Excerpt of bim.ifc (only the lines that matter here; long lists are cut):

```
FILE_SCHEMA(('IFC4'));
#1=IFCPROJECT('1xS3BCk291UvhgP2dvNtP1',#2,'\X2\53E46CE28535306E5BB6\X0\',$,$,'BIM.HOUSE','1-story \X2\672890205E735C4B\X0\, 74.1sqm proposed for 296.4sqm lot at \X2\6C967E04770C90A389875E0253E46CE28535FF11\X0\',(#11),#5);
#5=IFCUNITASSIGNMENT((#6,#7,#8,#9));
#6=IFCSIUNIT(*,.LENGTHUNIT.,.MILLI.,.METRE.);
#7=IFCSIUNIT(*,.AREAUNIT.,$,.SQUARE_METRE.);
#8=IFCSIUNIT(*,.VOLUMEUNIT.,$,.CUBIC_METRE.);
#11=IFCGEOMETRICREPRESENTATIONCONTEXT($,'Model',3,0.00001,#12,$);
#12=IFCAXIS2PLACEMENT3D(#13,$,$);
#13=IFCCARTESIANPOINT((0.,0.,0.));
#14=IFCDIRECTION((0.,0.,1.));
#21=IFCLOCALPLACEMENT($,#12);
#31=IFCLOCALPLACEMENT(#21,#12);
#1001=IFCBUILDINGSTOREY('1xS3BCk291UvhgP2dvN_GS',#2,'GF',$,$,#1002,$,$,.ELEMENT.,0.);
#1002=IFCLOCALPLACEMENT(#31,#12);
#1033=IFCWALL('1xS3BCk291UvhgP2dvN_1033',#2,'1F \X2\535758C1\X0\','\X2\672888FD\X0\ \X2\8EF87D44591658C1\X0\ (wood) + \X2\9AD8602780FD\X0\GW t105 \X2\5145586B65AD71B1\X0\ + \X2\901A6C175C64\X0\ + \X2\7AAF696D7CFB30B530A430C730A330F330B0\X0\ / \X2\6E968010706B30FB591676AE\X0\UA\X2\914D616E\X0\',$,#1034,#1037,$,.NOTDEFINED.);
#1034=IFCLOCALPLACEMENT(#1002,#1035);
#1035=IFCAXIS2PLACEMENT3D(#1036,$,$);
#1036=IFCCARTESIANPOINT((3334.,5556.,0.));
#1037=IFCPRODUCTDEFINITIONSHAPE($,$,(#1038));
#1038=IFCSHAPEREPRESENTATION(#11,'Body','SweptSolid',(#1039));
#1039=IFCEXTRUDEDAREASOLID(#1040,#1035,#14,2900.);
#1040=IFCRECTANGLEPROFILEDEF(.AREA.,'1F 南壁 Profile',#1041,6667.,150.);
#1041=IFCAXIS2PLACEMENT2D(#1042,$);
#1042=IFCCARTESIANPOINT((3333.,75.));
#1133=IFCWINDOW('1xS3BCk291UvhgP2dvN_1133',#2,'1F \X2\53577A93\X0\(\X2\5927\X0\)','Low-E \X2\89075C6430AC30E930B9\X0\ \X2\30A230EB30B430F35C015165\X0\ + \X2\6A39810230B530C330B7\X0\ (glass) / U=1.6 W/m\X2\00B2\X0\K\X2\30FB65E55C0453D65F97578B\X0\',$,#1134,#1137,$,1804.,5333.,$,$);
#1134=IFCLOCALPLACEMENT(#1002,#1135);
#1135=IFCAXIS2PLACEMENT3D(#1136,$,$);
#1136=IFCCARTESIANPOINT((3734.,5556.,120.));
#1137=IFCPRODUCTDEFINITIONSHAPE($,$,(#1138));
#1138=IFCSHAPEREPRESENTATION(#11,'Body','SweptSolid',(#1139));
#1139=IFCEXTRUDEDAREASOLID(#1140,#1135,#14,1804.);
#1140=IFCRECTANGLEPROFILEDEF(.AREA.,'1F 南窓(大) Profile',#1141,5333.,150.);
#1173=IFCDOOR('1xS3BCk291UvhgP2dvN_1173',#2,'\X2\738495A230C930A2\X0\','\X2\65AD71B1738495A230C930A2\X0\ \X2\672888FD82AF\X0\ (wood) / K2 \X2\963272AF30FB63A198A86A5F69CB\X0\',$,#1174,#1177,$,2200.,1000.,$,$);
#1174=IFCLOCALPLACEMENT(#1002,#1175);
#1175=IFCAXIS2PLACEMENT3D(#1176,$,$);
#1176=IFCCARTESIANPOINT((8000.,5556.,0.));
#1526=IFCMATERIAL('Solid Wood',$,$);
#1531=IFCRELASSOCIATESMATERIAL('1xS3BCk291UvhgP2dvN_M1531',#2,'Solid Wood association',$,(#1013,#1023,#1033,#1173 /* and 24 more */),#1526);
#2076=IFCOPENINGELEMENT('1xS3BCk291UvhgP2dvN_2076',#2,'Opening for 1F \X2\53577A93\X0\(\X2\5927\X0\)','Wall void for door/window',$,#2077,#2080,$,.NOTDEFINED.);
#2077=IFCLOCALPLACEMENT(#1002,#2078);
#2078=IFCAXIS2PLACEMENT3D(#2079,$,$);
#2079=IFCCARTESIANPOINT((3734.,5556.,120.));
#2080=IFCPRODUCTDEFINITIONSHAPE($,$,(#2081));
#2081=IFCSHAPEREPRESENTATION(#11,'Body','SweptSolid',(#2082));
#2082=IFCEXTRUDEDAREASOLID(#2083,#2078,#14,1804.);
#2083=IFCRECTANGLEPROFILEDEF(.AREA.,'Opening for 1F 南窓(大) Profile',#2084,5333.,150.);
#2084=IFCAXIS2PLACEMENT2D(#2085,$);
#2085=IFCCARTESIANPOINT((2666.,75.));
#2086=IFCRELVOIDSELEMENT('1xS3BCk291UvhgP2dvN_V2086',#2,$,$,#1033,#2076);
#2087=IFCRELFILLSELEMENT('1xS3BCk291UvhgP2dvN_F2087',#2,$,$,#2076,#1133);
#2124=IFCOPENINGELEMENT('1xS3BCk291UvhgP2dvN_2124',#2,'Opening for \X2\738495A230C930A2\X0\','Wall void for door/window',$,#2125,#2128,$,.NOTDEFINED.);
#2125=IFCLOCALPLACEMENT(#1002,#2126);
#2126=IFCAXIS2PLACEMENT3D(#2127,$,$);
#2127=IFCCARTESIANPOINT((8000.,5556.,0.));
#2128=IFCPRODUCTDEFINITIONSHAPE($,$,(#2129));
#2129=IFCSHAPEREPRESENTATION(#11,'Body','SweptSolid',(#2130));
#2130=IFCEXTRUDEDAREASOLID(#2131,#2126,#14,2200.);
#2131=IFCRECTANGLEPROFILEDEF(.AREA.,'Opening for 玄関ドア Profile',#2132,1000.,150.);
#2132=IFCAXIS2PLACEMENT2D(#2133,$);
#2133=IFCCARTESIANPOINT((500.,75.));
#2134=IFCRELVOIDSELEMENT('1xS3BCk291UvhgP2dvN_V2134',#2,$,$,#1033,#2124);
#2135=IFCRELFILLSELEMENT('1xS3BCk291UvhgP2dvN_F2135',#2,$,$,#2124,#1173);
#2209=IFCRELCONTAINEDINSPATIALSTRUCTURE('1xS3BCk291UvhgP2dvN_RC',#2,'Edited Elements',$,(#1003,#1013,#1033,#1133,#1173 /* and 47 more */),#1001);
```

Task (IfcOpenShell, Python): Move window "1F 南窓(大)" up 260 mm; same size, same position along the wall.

```python
import numpy as np
import ifcopenshell
import ifcopenshell.api.geometry
import ifcopenshell.util.placement
import ifcopenshell.util.unit

model = ifcopenshell.open("bim.ifc")
unit_scale = ifcopenshell.util.unit.calculate_unit_scale(model)

window = model.by_guid("1xS3BCk291UvhgP2dvN_1133")
opening = window.FillsVoids[0].RelatingOpeningElement
dz = 260.0

shift = np.array([0.0, 0.0, dz])
# The window is not placed relative to its opening, so move both.
for product in (opening, window):
    matrix = ifcopenshell.util.placement.get_local_placement(product.ObjectPlacement)
    matrix[:3, 3] += shift
    ifcopenshell.api.geometry.edit_object_placement(model, product=product, matrix=matrix, is_si=False)

print(f"moved by {dz * unit_scale:+.3f} m")

model.write("bim-out.ifc")
```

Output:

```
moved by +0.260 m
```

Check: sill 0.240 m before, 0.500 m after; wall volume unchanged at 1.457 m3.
